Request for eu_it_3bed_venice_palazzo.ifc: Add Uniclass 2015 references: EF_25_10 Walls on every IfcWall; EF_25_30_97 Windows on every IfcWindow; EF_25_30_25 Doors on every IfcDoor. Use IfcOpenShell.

First a look at what the model holds.

```python
import ifcopenshell

model = ifcopenshell.open("eu_it_3bed_venice_palazzo.ifc")
print(model.schema)
print("classifications:", [c.Name for c in model.by_type("IfcClassification")])
for ifc_class in ("IfcDoor", "IfcRoof", "IfcStair", "IfcWall", "IfcWindow"):
    print(ifc_class, len(model.by_type(ifc_class)))
```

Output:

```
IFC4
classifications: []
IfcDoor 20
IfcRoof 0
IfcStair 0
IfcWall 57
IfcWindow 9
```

```python
import ifcopenshell
import ifcopenshell.api.classification

model = ifcopenshell.open("eu_it_3bed_venice_palazzo.ifc")

system = ifcopenshell.api.classification.add_classification(model, classification="Uniclass 2015")

codes = {
    "IfcWall": ("EF_25_10", "Walls"),
    "IfcWindow": ("EF_25_30_97", "Windows"),
    "IfcDoor": ("EF_25_30_25", "Doors"),
}
for ifc_class, (code, name) in codes.items():
    products = model.by_type(ifc_class)
    ifcopenshell.api.classification.add_reference(
        model, products=products, classification=system, identification=code, name=name
    )
    print(code, len(products))

model.write("eu_it_3bed_venice_palazzo-out.ifc")
```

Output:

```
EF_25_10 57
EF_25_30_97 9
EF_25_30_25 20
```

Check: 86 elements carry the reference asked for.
